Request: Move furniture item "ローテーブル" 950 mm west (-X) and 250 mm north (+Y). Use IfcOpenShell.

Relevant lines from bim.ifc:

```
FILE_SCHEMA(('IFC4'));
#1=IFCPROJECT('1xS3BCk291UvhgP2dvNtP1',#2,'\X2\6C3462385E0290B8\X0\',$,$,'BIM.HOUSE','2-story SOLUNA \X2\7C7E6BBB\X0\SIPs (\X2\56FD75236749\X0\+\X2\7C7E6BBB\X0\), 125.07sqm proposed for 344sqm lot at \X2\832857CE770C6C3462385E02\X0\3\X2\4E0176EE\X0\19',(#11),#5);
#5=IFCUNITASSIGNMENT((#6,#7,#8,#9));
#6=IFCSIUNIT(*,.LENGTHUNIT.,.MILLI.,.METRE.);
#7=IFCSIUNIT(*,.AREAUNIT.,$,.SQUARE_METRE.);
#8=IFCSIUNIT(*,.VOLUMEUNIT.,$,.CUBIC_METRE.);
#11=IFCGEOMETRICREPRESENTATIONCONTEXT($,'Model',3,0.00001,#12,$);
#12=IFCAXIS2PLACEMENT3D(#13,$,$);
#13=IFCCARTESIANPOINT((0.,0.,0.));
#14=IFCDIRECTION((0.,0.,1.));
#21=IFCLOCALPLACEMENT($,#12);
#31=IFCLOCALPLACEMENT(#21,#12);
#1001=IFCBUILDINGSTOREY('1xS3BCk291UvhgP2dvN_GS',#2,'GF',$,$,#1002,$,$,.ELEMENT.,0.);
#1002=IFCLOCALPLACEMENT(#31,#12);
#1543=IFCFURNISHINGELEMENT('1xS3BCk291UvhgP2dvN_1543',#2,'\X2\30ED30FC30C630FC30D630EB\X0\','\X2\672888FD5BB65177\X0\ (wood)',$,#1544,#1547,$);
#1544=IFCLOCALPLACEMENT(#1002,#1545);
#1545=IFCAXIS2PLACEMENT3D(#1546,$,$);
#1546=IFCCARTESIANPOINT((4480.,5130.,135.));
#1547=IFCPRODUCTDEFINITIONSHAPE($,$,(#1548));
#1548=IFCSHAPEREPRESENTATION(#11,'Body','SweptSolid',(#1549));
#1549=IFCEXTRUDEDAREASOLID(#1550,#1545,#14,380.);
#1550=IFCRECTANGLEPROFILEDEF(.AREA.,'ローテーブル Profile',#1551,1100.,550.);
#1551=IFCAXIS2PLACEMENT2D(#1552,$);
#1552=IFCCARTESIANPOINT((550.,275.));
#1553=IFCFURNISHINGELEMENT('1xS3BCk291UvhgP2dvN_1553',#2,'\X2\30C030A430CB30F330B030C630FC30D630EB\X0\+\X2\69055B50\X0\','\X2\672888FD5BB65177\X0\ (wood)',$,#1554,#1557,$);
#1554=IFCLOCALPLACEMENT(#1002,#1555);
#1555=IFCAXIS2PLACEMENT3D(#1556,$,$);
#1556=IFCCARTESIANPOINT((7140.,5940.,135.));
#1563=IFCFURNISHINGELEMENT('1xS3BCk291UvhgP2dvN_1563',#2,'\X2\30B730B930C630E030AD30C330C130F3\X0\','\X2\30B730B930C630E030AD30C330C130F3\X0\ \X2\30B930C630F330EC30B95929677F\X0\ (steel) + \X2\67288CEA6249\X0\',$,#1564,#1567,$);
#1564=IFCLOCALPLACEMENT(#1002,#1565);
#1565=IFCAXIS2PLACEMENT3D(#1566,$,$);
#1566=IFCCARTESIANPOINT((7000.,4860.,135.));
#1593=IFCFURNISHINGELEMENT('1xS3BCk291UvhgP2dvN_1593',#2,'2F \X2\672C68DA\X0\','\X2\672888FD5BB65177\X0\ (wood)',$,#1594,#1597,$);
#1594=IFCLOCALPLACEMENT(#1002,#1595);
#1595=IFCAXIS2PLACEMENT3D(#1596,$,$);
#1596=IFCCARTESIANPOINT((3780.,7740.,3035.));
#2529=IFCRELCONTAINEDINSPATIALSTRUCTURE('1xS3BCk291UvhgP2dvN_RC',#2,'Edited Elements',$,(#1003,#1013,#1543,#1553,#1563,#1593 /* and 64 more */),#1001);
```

```python
import ifcopenshell
import ifcopenshell.api.geometry
import ifcopenshell.util.placement

model = ifcopenshell.open("bim.ifc")

item = model.by_guid("1xS3BCk291UvhgP2dvN_1543")
matrix = ifcopenshell.util.placement.get_local_placement(item.ObjectPlacement)
matrix[0, 3] -= 950.0
matrix[1, 3] += 250.0
ifcopenshell.api.geometry.edit_object_placement(model, product=item, matrix=matrix, is_si=False)

print(ifcopenshell.util.placement.get_local_placement(item.ObjectPlacement).round(3) + 0.0)

model.write("bim_v2.ifc")
```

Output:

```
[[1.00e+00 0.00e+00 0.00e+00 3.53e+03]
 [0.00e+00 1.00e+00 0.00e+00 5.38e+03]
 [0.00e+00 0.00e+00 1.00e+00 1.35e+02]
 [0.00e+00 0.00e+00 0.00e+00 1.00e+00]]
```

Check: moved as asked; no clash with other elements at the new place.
